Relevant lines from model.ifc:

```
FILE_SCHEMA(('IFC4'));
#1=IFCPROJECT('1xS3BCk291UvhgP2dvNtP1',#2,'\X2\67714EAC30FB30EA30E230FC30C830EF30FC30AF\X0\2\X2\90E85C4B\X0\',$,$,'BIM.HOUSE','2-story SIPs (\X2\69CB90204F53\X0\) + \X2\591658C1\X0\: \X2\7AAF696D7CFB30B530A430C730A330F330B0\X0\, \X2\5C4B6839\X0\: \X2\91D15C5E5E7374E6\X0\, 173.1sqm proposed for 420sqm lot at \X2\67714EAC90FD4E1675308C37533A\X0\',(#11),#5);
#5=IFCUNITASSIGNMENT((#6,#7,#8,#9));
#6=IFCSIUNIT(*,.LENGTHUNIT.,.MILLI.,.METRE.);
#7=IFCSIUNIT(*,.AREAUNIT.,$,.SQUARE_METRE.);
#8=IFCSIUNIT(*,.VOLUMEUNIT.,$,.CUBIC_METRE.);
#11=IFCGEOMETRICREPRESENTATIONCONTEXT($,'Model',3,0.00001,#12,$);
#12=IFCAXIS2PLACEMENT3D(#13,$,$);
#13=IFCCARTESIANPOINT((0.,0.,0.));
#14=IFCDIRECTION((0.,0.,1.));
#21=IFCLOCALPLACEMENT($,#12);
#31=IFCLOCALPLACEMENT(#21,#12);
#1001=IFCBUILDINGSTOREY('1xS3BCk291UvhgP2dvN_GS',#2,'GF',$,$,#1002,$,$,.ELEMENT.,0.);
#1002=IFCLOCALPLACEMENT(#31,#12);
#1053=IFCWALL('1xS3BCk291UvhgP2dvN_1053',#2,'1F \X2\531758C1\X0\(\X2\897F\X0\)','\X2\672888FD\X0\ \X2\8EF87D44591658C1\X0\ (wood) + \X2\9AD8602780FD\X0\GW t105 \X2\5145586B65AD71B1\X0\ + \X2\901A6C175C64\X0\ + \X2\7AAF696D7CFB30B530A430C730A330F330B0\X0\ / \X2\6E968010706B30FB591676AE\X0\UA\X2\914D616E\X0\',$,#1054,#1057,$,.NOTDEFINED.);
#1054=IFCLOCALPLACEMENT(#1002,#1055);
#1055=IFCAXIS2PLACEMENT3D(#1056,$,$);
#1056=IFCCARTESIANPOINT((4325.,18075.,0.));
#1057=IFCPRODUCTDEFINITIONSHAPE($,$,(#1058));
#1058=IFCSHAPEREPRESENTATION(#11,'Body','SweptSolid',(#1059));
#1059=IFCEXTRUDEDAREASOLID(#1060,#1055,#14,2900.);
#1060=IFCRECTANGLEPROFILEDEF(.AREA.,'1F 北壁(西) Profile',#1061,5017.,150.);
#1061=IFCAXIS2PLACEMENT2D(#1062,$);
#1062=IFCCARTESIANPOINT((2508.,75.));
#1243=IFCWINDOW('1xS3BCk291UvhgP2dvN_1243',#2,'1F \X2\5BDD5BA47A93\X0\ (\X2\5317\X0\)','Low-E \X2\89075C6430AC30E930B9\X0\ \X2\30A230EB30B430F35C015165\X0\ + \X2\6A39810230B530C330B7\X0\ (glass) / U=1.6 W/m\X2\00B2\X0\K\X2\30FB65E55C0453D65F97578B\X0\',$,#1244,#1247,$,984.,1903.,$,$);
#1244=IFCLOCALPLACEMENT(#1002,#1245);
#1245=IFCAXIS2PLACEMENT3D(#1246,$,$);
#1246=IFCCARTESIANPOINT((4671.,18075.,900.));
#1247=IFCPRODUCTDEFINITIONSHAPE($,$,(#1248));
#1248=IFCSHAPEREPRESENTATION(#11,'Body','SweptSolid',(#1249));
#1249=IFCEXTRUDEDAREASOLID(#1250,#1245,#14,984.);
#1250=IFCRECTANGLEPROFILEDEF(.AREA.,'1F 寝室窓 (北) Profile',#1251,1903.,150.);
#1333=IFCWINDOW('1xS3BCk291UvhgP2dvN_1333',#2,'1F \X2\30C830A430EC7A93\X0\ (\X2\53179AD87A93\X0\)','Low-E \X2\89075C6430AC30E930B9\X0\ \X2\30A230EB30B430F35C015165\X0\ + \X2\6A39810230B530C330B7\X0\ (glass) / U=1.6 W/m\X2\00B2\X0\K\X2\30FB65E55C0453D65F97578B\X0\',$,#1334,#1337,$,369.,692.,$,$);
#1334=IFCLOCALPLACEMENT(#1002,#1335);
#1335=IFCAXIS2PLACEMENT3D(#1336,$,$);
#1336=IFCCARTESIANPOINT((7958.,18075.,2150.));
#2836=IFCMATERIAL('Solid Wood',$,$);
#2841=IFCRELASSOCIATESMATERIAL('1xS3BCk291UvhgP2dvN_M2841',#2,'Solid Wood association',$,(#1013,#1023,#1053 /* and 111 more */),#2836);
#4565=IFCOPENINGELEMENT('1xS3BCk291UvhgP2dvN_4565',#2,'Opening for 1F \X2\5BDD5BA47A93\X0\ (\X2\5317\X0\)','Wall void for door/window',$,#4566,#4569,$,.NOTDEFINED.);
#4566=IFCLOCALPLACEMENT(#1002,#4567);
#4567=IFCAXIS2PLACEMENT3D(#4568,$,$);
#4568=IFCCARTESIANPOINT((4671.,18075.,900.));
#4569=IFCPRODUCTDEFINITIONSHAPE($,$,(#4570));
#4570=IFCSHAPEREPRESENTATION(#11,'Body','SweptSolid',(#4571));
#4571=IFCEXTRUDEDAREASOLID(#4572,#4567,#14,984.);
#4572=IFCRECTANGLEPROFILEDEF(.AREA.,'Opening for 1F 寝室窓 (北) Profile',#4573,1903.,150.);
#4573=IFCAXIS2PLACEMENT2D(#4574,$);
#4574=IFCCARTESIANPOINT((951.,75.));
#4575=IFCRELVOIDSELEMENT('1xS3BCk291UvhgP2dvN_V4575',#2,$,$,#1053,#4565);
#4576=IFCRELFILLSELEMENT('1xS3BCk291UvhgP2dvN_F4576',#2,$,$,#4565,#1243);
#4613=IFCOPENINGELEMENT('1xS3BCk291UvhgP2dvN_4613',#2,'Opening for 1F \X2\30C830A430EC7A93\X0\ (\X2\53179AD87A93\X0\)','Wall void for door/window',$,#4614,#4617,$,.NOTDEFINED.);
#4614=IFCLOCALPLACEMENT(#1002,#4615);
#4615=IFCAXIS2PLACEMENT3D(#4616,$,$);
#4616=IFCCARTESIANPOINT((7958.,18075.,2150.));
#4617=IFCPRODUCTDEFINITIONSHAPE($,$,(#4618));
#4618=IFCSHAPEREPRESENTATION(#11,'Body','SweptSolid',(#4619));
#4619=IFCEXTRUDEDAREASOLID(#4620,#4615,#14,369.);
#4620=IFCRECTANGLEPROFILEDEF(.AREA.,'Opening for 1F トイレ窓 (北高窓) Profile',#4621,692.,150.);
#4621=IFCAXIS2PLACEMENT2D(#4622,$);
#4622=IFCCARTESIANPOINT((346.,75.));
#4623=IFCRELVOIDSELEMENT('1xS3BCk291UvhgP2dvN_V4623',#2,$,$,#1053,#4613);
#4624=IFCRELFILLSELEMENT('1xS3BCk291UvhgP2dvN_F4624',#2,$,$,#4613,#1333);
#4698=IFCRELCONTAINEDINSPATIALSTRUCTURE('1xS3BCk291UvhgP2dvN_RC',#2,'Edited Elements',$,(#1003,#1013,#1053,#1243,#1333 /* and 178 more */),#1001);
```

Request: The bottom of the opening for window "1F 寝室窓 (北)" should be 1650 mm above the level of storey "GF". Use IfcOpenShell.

```python
import numpy as np
import ifcopenshell
import ifcopenshell.api.geometry
import ifcopenshell.geom
import ifcopenshell.util.element
import ifcopenshell.util.placement
import ifcopenshell.util.shape
import ifcopenshell.util.unit

model = ifcopenshell.open("model.ifc")
unit_scale = ifcopenshell.util.unit.calculate_unit_scale(model)

window = model.by_id(1243)
opening = window.FillsVoids[0].RelatingOpeningElement
storey = ifcopenshell.util.element.get_container(window, ifc_class="IfcBuildingStorey")
level = ifcopenshell.util.placement.get_local_placement(storey.ObjectPlacement)[2, 3]

# The opening's origin need not be at the sill, so measure its lowest point.
shape = ifcopenshell.geom.create_shape(ifcopenshell.geom.settings(), opening)
bottom = ifcopenshell.util.shape.get_shape_bottom_elevation(shape, shape.geometry) / unit_scale
dz = level + 1.65 / unit_scale - bottom

shift = np.array([0.0, 0.0, dz])
# The window is not placed relative to its opening, so move both.
for product in (opening, window):
    matrix = ifcopenshell.util.placement.get_local_placement(product.ObjectPlacement)
    matrix[:3, 3] += shift
    ifcopenshell.api.geometry.edit_object_placement(model, product=product, matrix=matrix, is_si=False)

print(f"moved by {dz * unit_scale:+.3f} m")

model.write("model_updated.ifc")
```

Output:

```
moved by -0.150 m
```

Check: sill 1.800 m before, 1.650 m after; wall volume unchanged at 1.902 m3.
